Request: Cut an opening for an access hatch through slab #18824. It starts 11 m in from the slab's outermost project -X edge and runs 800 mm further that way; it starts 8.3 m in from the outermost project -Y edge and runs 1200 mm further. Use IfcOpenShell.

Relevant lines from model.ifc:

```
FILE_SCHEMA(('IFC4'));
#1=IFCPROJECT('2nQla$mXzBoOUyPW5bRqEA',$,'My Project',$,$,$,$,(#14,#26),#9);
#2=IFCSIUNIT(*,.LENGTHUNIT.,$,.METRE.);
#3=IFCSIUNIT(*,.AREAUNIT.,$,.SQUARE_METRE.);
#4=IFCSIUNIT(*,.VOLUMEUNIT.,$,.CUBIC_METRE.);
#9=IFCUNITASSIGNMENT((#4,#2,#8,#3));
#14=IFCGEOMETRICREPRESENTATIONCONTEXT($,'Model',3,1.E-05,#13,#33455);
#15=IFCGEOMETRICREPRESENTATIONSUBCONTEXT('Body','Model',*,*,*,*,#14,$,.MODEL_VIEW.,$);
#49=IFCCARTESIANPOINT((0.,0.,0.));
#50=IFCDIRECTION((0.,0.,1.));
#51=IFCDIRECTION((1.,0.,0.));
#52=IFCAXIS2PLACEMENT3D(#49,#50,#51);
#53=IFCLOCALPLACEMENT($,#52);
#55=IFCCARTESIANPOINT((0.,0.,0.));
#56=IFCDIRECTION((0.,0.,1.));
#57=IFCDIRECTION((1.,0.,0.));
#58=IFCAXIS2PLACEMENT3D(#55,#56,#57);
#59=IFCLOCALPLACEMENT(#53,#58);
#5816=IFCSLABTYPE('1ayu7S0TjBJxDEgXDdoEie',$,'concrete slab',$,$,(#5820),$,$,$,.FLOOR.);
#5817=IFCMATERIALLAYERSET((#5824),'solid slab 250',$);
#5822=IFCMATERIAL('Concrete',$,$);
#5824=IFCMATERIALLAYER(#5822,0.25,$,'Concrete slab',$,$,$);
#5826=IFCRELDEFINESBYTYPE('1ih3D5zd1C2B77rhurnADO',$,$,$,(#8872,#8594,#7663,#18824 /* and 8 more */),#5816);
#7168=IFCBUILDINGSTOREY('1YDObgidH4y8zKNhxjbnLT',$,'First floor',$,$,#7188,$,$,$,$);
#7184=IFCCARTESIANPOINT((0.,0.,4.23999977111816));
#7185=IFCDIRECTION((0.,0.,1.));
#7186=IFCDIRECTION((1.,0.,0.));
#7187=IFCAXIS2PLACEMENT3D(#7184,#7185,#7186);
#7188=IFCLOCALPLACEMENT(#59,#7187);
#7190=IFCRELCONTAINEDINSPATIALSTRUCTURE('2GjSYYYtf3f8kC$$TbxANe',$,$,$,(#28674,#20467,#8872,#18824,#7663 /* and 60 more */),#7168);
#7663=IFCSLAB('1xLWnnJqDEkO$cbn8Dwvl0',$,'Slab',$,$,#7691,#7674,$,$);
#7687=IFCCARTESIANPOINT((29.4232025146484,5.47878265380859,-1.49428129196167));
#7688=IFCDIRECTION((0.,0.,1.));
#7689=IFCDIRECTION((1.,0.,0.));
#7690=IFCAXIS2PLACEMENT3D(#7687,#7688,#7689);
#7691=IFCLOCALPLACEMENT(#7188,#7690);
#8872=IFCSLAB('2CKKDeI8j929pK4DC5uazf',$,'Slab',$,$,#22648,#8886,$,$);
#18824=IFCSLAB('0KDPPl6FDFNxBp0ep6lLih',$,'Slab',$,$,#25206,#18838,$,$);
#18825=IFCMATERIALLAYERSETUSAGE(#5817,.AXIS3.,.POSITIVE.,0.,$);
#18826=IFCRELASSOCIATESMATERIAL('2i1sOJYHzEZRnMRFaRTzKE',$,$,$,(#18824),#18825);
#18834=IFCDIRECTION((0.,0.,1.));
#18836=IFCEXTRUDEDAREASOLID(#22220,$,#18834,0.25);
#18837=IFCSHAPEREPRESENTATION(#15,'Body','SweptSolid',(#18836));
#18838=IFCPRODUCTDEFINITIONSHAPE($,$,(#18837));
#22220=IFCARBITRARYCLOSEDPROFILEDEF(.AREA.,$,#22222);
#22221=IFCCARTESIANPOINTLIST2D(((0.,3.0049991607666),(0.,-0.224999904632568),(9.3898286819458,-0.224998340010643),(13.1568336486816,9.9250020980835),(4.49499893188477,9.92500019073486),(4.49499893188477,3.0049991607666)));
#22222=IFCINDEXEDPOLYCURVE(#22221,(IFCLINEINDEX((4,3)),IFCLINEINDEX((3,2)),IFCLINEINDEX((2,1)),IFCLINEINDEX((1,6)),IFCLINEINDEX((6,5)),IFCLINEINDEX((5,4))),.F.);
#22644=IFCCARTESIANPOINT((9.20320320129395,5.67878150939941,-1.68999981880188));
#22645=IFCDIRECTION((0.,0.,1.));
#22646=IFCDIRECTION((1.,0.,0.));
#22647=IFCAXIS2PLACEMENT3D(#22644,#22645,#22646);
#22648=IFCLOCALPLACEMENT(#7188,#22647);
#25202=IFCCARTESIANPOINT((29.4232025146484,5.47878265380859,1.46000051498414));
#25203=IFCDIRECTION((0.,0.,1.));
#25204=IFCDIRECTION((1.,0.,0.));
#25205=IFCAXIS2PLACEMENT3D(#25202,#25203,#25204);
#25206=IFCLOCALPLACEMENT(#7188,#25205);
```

```python
import numpy as np
import ifcopenshell
import ifcopenshell.api.feature
import ifcopenshell.api.geometry
import ifcopenshell.api.root
import ifcopenshell.geom
import ifcopenshell.util.placement
import ifcopenshell.util.representation
import ifcopenshell.util.shape
import ifcopenshell.util.unit

model = ifcopenshell.open("model.ifc")
unit_scale = ifcopenshell.util.unit.calculate_unit_scale(model)
settings = ifcopenshell.geom.settings()


def volume(element):
    """Net volume in cubic metres, openings subtracted."""
    shape = ifcopenshell.geom.create_shape(settings, element)
    return ifcopenshell.util.shape.get_volume(shape.geometry)


slab = model.by_guid("0KDPPl6FDFNxBp0ep6lLih")
before = volume(slab)

# Extent in the slab's own axes, in metres. The edges named are its -X and -Y sides.
slab_shape = ifcopenshell.geom.create_shape(settings, slab)
vertices = ifcopenshell.util.shape.get_vertices(slab_shape.geometry)
x_min, y_min, bottom = vertices.min(axis=0)
top = vertices[:, 2].max()

opening = ifcopenshell.api.root.create_entity(model, ifc_class="IfcOpeningElement", name="Access hatch opening", predefined_type="OPENING")
context = ifcopenshell.util.representation.get_context(model, "Model", "Body", "MODEL_VIEW")
width, depth = 0.8, 1.2
outline = [(0.0, 0.0), (width, 0.0), (width, depth), (0.0, depth), (0.0, 0.0)]
# Overshoot both faces by 50 mm so the cut is clean.
shape = ifcopenshell.api.geometry.add_slab_representation(
    model, context=context, depth=top - bottom + 0.1, polyline=outline
)
ifcopenshell.api.geometry.assign_representation(model, product=opening, representation=shape)

matrix = ifcopenshell.util.placement.get_local_placement(slab.ObjectPlacement)
matrix[:, 3] = matrix @ np.append(np.array([x_min + 11, y_min + 8.3, bottom - 0.05]) / unit_scale, 1.0)
ifcopenshell.api.geometry.edit_object_placement(model, product=opening, matrix=matrix, is_si=False)
ifcopenshell.api.feature.add_feature(model, feature=opening, element=slab)

after = volume(slab)

print(f"slab volume {before:.3f} -> {after:.3f} m3")

model.write("model_updated.ifc")
```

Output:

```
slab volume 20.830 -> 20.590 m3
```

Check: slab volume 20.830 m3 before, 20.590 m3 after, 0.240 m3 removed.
